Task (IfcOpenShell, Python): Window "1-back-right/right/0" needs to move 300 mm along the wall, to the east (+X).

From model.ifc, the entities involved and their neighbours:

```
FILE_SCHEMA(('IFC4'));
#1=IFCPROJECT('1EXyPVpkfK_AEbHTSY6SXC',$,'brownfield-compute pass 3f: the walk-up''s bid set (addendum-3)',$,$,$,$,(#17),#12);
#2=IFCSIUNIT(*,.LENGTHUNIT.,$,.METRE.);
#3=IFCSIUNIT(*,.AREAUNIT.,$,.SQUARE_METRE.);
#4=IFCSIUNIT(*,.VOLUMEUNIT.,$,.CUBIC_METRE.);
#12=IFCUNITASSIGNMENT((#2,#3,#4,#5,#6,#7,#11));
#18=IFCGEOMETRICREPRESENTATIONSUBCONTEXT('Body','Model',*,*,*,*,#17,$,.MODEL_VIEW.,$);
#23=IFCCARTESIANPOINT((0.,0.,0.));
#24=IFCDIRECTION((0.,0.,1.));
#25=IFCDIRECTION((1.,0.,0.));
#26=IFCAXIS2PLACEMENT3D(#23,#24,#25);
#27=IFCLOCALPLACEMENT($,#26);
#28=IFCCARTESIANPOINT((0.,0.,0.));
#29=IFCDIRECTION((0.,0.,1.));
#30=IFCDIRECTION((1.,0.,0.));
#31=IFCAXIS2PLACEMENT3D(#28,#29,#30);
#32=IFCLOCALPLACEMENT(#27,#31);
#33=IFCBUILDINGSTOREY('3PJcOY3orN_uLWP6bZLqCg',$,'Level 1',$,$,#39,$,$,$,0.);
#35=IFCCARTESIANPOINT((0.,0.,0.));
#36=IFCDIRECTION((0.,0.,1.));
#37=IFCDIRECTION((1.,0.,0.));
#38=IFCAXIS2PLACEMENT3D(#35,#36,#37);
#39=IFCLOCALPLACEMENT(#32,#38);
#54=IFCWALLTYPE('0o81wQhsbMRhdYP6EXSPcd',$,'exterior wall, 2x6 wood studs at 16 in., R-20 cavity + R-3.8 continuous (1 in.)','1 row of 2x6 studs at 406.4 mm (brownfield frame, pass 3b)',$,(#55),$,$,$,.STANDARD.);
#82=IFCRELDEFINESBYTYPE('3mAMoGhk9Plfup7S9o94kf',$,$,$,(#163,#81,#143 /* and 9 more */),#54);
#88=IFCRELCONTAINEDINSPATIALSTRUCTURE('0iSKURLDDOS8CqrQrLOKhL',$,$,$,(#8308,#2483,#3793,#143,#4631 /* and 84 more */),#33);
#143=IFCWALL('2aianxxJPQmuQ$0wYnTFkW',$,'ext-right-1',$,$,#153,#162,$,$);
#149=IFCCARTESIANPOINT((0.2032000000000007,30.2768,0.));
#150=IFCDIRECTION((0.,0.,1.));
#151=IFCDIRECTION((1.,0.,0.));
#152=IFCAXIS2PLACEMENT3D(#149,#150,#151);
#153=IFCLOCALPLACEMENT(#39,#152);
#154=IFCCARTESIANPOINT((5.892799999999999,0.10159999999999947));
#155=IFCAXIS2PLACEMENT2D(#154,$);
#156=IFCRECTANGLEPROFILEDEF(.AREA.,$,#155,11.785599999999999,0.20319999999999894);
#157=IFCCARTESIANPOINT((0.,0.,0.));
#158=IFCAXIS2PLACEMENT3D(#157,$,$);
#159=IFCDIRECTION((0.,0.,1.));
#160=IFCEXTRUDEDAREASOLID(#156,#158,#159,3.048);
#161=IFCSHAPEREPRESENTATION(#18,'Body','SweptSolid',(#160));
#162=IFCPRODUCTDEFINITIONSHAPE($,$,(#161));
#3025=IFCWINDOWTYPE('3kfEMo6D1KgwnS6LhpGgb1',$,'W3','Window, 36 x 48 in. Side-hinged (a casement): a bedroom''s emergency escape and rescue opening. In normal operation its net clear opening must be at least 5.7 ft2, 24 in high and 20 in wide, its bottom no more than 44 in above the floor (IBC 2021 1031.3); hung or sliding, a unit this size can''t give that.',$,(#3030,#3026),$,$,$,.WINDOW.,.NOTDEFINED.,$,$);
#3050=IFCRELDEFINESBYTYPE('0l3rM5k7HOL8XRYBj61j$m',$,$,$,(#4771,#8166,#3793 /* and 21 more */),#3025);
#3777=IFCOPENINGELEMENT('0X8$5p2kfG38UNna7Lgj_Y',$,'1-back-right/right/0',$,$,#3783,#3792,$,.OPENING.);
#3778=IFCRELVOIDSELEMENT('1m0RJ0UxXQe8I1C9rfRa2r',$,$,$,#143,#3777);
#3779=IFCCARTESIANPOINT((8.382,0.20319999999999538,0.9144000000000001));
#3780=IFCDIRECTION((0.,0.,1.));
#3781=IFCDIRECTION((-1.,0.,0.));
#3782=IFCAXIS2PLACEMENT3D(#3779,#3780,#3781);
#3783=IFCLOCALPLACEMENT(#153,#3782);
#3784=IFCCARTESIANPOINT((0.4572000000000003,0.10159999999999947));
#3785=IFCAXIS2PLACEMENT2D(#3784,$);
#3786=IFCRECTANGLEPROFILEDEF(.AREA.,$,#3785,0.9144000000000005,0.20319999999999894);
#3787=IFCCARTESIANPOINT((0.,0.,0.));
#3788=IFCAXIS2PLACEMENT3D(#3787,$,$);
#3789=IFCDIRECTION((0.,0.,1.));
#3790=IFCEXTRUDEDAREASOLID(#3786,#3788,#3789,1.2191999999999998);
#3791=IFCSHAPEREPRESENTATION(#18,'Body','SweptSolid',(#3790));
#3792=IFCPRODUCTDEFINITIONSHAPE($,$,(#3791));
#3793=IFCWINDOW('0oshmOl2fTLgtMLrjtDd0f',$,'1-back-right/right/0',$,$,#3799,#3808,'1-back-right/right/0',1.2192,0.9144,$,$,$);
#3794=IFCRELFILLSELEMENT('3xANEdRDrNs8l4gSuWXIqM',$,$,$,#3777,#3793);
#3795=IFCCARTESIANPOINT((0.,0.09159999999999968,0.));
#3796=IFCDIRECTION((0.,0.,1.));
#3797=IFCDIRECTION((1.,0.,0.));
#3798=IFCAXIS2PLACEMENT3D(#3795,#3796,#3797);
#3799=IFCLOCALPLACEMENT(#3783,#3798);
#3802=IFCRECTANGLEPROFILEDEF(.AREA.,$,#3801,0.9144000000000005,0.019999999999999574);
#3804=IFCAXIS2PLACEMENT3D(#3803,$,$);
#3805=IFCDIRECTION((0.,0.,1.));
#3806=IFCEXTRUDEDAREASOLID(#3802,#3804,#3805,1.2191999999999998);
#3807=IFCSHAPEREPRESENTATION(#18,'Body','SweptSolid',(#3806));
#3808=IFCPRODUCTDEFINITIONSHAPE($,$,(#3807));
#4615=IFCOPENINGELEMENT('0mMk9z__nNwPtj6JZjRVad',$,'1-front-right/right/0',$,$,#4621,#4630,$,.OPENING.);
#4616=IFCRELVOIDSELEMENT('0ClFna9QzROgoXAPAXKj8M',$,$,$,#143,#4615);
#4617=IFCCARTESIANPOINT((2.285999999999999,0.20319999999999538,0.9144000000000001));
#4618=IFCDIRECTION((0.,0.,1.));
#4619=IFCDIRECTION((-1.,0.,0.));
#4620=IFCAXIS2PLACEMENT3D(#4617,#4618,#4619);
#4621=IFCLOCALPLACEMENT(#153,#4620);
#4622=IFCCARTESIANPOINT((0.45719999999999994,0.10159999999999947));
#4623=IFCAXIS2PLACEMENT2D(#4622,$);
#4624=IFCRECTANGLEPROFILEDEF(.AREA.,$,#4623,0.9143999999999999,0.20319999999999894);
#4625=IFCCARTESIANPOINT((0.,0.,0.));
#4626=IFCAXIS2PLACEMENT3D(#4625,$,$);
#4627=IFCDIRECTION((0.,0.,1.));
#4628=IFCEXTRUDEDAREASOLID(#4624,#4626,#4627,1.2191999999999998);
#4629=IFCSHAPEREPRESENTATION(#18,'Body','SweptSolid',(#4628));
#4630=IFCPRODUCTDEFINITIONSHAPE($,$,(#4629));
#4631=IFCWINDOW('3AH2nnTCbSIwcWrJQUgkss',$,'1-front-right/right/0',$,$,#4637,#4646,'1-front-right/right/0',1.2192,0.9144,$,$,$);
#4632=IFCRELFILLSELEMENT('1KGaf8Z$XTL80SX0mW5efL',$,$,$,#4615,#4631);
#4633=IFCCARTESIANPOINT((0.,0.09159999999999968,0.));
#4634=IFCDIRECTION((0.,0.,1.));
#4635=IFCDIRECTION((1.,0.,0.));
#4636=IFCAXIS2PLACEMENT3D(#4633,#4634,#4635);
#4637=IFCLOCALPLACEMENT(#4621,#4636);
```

```python
import ifcopenshell
import ifcopenshell.api.geometry
import ifcopenshell.util.placement

model = ifcopenshell.open("model.ifc")

window = model.by_id(3793)
opening = window.FillsVoids[0].RelatingOpeningElement
wall = opening.VoidsElements[0].RelatingBuildingElement

wall_matrix = ifcopenshell.util.placement.get_local_placement(wall.ObjectPlacement)
shift = wall_matrix[:3, 0] * 0.3
before = ifcopenshell.util.placement.get_local_placement(window.ObjectPlacement)[:3, 3].copy()

# The window is placed relative to its opening, so it follows when the opening moves.
matrix = ifcopenshell.util.placement.get_local_placement(opening.ObjectPlacement)
matrix[:3, 3] += shift
ifcopenshell.api.geometry.edit_object_placement(
    model, product=opening, matrix=matrix, is_si=False, should_transform_children=True
)

after = ifcopenshell.util.placement.get_local_placement(window.ObjectPlacement)[:3, 3]
print("window moved by", (after - before).round(3) + 0.0)

model.write("model_updated.ifc")
```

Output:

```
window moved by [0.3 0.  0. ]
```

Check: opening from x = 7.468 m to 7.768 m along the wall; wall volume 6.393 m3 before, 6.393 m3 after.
